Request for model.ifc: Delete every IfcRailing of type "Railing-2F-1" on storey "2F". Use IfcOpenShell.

First a look at what the model holds.

```python
import ifcopenshell
import ifcopenshell.util.element

model = ifcopenshell.open("model.ifc")
print(model.schema)
storey = next(s for s in model.by_type("IfcBuildingStorey") if s.Name == "2F")
railings = [e for e in ifcopenshell.util.element.get_decomposition(storey) if e.is_a("IfcRailing")]
seen = {}
for e in railings:
    element_type = ifcopenshell.util.element.get_type(e)
    name = element_type.Name if element_type not in (None, e) else None
    seen[name] = seen.get(name, 0) + 1
for name, count in sorted(seen.items(), key=str):
    print(count, "x", name)
```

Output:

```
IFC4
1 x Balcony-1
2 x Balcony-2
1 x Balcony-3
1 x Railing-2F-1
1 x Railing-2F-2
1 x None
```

```python
import ifcopenshell
import ifcopenshell.api.root
import ifcopenshell.util.element

model = ifcopenshell.open("model.ifc")

storey = next(s for s in model.by_type("IfcBuildingStorey") if s.Name == "2F")
railings = [e for e in ifcopenshell.util.element.get_decomposition(storey) if e.is_a("IfcRailing")]
targets = [e for e in railings if (t := ifcopenshell.util.element.get_type(e)) not in (None, e) and t.Name == "Railing-2F-1"]

for e in targets:
    ifcopenshell.api.root.remove_product(model, product=e)
print(len(targets), "removed")

model.write("model-out.ifc")
```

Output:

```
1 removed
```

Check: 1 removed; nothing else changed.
